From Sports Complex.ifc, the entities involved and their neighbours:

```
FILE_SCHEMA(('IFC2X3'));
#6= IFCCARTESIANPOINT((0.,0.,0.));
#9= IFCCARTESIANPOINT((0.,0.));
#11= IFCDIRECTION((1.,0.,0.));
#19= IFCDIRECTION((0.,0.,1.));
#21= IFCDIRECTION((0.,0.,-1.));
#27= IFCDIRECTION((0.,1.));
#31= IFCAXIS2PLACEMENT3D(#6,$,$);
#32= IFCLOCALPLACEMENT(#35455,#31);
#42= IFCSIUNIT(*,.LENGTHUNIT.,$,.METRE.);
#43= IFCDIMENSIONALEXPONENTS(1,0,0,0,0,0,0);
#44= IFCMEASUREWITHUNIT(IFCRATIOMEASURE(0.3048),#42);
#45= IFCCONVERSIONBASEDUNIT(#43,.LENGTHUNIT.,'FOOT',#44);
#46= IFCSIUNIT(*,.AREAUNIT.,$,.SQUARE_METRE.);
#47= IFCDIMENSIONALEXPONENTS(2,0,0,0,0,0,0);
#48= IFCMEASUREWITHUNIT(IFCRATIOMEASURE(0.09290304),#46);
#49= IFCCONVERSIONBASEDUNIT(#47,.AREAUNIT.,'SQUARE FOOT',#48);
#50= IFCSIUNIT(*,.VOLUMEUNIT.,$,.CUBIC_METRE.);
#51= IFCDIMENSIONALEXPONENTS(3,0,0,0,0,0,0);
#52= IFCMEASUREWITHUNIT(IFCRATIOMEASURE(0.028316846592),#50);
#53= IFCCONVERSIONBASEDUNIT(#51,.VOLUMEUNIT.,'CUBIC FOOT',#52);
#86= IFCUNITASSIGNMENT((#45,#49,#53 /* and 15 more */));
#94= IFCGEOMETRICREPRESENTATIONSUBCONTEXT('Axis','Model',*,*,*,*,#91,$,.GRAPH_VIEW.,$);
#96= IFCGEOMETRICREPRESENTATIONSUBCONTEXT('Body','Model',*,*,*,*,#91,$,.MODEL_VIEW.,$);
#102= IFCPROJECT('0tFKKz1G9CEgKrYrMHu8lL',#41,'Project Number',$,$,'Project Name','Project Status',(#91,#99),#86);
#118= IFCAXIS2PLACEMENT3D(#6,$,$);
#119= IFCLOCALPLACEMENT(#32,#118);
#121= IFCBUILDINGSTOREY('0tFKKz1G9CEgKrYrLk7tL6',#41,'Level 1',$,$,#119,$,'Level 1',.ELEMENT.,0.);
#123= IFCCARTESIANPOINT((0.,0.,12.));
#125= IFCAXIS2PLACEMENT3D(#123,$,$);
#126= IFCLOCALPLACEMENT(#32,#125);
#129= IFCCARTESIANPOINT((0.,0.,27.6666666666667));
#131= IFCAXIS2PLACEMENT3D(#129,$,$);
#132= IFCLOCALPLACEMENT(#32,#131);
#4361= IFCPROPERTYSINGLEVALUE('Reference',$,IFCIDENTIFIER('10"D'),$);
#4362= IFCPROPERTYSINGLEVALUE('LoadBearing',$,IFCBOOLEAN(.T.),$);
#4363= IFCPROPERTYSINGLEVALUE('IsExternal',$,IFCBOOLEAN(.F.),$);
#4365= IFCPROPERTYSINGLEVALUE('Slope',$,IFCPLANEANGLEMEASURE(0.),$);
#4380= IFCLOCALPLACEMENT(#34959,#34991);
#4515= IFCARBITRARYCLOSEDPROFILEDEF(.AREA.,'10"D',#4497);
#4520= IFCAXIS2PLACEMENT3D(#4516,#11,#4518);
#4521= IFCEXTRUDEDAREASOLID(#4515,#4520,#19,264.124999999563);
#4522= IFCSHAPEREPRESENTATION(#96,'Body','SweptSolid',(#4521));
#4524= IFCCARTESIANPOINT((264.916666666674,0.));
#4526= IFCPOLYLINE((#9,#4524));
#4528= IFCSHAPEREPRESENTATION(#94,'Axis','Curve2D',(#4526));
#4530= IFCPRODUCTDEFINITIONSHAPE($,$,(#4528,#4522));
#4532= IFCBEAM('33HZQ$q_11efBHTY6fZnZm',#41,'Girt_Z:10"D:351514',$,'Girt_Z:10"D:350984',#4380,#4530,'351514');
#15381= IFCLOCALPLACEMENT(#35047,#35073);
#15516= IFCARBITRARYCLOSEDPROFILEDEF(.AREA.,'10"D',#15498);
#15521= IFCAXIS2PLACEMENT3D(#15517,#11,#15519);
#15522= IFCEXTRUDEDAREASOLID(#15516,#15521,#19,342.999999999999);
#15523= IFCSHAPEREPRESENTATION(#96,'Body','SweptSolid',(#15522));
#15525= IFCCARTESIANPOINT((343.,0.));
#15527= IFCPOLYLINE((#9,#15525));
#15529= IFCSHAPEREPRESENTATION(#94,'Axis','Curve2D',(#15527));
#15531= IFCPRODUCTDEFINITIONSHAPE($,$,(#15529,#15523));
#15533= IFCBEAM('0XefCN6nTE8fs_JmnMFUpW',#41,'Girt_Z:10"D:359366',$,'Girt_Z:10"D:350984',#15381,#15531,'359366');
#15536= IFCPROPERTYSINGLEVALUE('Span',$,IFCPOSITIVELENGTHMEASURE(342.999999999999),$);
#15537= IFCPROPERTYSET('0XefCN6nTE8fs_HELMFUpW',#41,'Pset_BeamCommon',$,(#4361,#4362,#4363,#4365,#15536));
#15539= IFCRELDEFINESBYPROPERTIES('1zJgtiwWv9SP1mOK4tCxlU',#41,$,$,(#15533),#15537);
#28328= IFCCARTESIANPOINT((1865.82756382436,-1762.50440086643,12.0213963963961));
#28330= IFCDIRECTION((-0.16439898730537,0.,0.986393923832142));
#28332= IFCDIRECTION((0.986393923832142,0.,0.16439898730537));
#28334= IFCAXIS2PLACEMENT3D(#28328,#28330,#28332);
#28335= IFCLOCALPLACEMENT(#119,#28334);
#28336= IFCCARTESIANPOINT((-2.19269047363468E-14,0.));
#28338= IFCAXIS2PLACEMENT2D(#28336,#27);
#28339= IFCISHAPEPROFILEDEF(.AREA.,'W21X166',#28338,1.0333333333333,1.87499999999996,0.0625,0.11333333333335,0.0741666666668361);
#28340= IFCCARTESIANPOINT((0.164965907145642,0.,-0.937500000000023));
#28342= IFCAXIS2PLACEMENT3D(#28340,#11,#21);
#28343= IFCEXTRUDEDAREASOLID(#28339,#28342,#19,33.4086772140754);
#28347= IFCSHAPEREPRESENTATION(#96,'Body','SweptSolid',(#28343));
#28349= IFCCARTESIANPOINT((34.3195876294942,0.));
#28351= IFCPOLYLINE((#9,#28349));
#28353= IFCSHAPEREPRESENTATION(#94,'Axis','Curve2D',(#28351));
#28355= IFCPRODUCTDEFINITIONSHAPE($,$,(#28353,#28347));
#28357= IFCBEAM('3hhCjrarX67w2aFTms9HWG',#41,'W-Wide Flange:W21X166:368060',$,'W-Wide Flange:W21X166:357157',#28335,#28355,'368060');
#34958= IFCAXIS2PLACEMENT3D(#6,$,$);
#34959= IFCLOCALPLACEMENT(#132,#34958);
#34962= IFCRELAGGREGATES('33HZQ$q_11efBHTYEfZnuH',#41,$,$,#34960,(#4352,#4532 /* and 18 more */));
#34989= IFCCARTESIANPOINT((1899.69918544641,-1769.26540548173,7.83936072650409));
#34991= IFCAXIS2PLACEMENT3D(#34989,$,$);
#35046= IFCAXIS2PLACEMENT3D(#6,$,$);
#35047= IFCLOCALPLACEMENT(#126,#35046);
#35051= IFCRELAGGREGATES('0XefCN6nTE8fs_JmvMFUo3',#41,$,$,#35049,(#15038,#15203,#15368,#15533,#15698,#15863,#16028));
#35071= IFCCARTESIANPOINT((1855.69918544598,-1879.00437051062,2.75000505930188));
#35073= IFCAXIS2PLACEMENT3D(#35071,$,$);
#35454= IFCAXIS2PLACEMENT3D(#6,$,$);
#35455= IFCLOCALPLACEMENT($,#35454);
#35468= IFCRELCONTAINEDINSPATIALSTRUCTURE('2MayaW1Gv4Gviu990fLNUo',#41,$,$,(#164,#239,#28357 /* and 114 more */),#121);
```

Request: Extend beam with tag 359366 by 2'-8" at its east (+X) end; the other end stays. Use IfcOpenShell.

```python
import numpy as np
import ifcopenshell
import ifcopenshell.api.pset
import ifcopenshell.util.element
import ifcopenshell.util.representation
import ifcopenshell.util.unit

model = ifcopenshell.open("Sports Complex.ifc")
unit_scale = ifcopenshell.util.unit.calculate_unit_scale(model)

member = model.by_id(15533)
change = 32 * 0.0254 / unit_scale

# The extrusion runs towards the end named, so only its depth changes.
body = ifcopenshell.util.representation.get_representation(member, "Model", "Body")
solid = body.Items[0]
old_length = solid.Depth
solid.Depth += change

# Move the axis end point with it.
axis = next(r for r in member.Representation.Representations if r.RepresentationIdentifier == "Axis").Items[0]
start, end = (np.array(p.Coordinates) for p in axis.Points)
end = end + (end - start) / np.linalg.norm(end - start) * change
point = model.createIfcCartesianPoint(end.tolist())
axis.Points = [axis.Points[0], point]

# Update the stored length and volume.
pset = model.by_id(ifcopenshell.util.element.get_pset(member, "Pset_BeamCommon", should_inherit=False)["id"])
ifcopenshell.api.pset.edit_pset(model, pset=pset, properties={
    "Span": model.create_entity("IfcPositiveLengthMeasure", solid.Depth),
})

print(f"length {old_length:g} -> {solid.Depth:g}")

model.write("Sports Complex_rev.ifc")
```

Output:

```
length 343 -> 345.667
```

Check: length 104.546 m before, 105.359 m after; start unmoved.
